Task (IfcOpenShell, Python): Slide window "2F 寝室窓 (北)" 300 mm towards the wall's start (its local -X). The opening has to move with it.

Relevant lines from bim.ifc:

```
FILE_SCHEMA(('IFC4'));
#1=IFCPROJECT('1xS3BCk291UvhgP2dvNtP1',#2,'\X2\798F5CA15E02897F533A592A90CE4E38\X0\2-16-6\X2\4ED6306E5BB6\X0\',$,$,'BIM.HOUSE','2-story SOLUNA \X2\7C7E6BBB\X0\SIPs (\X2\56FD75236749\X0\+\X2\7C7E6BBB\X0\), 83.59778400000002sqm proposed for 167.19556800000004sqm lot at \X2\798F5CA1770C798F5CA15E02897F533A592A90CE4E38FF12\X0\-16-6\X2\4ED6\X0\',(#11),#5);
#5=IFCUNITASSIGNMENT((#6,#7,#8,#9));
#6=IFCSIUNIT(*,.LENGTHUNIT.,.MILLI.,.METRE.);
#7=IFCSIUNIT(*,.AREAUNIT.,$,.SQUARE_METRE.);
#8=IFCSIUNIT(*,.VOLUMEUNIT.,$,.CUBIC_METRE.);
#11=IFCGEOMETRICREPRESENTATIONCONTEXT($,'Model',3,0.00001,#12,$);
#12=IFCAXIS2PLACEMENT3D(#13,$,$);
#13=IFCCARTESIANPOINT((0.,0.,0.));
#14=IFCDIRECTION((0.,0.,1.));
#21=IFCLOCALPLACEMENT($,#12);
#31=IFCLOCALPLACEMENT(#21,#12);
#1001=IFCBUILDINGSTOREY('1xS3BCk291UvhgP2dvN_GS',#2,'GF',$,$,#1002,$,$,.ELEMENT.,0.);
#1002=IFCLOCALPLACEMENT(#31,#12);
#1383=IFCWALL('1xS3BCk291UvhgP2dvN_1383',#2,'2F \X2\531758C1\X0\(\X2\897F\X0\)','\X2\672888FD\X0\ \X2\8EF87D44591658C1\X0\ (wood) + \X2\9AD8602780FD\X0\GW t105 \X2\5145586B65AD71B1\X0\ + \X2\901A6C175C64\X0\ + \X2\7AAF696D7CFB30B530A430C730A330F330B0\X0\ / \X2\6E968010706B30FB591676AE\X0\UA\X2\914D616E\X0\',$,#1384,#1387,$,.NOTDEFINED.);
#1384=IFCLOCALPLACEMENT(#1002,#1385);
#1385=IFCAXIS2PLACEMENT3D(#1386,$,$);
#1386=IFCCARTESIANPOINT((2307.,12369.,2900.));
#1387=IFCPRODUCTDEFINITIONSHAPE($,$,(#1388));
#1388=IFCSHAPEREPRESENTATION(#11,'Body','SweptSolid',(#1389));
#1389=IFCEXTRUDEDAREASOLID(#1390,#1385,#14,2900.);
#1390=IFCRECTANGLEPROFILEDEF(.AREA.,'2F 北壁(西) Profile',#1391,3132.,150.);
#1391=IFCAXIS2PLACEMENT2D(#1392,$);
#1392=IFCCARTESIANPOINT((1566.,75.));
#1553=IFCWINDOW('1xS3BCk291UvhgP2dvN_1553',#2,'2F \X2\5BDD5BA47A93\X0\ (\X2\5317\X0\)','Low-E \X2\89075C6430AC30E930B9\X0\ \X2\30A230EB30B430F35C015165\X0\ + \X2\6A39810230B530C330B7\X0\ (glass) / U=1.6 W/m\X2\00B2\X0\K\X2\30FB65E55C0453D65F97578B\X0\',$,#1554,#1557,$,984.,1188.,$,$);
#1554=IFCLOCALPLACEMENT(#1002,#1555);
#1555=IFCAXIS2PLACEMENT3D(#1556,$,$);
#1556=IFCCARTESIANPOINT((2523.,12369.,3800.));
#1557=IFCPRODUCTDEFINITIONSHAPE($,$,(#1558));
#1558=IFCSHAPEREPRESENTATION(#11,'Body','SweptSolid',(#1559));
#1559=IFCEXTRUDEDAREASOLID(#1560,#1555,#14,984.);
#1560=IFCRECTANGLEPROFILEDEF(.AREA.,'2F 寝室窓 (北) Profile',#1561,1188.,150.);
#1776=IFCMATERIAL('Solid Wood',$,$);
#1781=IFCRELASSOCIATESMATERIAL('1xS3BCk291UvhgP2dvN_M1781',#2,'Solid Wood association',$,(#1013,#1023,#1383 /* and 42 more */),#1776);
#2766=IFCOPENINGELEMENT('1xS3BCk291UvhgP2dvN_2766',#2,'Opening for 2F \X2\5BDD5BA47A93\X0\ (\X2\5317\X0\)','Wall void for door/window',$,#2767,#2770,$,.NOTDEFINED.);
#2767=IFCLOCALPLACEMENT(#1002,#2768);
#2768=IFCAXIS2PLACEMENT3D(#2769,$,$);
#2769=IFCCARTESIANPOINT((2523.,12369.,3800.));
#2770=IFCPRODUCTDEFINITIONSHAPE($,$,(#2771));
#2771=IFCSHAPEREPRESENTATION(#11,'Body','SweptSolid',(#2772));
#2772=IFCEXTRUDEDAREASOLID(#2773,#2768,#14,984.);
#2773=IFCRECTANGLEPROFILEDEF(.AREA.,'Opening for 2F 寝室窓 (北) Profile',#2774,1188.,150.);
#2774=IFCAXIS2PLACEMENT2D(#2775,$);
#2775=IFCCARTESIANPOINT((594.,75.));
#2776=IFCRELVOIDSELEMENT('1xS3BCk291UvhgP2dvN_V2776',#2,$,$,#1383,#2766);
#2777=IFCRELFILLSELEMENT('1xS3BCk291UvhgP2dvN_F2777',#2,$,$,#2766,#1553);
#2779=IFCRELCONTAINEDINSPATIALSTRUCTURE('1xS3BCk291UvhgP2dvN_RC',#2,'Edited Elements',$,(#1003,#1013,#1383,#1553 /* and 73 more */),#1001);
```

```python
import ifcopenshell
import ifcopenshell.api.geometry
import ifcopenshell.util.placement
import ifcopenshell.util.unit

model = ifcopenshell.open("bim.ifc")
unit_scale = ifcopenshell.util.unit.calculate_unit_scale(model)

window = model.by_guid("1xS3BCk291UvhgP2dvN_1553")
opening = window.FillsVoids[0].RelatingOpeningElement
wall = opening.VoidsElements[0].RelatingBuildingElement

wall_matrix = ifcopenshell.util.placement.get_local_placement(wall.ObjectPlacement)
shift = wall_matrix[:3, 0] * -0.3 / unit_scale
before = ifcopenshell.util.placement.get_local_placement(window.ObjectPlacement)[:3, 3].copy()

# The window is not placed relative to its opening, so move both.
for product in (opening, window):
    matrix = ifcopenshell.util.placement.get_local_placement(product.ObjectPlacement)
    matrix[:3, 3] += shift
    ifcopenshell.api.geometry.edit_object_placement(model, product=product, matrix=matrix, is_si=False)

after = ifcopenshell.util.placement.get_local_placement(window.ObjectPlacement)[:3, 3]
print("window moved by", (after - before).round(3) + 0.0)

model.write("bim_updated.ifc")
```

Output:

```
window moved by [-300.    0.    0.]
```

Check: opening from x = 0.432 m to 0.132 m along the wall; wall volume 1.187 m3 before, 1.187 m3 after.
